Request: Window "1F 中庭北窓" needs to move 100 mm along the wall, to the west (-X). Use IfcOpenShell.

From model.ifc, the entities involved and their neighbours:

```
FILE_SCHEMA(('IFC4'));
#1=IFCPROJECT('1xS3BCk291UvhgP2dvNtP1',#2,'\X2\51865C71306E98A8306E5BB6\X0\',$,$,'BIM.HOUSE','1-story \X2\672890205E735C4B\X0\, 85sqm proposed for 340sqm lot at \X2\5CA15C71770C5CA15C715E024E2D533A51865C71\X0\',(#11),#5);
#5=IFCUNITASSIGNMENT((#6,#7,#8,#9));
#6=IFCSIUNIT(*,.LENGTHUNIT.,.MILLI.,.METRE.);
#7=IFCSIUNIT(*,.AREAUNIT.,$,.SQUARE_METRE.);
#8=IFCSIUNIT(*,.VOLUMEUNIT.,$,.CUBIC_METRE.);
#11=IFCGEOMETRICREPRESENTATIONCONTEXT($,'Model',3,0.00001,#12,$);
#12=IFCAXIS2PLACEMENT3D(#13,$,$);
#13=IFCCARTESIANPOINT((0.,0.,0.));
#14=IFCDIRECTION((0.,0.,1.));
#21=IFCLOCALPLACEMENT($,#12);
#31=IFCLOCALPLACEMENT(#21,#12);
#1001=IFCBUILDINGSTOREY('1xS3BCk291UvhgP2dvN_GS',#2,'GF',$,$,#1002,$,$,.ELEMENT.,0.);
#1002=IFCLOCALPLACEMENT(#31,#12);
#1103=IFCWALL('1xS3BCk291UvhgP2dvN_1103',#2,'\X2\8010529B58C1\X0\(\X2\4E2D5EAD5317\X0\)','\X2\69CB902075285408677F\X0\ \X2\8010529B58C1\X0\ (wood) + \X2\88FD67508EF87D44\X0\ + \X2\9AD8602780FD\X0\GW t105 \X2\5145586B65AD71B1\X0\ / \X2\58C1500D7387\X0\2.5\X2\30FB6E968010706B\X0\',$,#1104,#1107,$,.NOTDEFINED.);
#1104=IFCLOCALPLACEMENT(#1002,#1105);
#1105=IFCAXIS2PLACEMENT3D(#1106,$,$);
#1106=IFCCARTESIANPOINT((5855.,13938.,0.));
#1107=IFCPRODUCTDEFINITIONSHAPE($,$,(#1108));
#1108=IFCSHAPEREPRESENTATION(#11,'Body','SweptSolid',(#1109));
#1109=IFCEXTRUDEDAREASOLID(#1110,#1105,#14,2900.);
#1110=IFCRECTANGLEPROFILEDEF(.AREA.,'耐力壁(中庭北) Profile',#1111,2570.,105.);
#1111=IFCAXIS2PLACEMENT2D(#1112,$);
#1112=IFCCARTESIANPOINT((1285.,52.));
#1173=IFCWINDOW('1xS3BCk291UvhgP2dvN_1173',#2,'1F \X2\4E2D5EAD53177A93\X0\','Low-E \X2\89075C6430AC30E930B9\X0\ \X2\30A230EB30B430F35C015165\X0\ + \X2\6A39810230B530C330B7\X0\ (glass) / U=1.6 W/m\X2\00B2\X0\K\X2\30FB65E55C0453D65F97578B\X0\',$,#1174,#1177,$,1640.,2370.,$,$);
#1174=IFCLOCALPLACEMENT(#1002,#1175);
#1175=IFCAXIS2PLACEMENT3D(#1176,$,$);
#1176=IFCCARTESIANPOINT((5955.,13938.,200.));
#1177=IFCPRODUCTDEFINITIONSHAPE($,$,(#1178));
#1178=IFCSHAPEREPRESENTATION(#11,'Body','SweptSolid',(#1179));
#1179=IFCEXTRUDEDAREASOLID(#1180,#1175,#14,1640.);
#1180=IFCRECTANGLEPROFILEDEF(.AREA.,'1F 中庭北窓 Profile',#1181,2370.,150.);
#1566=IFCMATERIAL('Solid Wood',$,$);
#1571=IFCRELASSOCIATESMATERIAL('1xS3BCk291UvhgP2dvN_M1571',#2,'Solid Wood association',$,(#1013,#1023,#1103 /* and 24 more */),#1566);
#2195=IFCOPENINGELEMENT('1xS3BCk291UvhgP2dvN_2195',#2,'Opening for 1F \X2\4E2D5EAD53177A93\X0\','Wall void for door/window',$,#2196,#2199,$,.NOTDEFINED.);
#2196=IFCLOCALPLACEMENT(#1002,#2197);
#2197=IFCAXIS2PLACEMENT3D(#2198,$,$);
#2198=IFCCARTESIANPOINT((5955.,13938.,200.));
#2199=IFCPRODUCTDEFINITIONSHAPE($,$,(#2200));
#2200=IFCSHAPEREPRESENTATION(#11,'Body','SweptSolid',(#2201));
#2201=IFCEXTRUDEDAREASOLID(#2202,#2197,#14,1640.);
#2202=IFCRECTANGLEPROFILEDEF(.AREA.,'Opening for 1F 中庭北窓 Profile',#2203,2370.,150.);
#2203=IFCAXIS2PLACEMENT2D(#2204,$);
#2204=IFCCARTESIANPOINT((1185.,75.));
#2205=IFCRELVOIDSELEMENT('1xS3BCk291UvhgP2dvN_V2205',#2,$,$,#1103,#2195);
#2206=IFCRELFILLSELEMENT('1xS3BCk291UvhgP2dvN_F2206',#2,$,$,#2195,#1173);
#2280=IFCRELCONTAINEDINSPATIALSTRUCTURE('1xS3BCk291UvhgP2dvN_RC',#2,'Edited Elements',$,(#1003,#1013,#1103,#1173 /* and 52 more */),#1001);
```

```python
import ifcopenshell
import ifcopenshell.api.geometry
import ifcopenshell.util.placement
import ifcopenshell.util.unit

model = ifcopenshell.open("model.ifc")
unit_scale = ifcopenshell.util.unit.calculate_unit_scale(model)

window = model.by_guid("1xS3BCk291UvhgP2dvN_1173")
opening = window.FillsVoids[0].RelatingOpeningElement
wall = opening.VoidsElements[0].RelatingBuildingElement

wall_matrix = ifcopenshell.util.placement.get_local_placement(wall.ObjectPlacement)
shift = wall_matrix[:3, 0] * -0.1 / unit_scale
before = ifcopenshell.util.placement.get_local_placement(window.ObjectPlacement)[:3, 3].copy()

# The window is not placed relative to its opening, so move both.
for product in (opening, window):
    matrix = ifcopenshell.util.placement.get_local_placement(product.ObjectPlacement)
    matrix[:3, 3] += shift
    ifcopenshell.api.geometry.edit_object_placement(model, product=product, matrix=matrix, is_si=False)

after = ifcopenshell.util.placement.get_local_placement(window.ObjectPlacement)[:3, 3]
print("window moved by", (after - before).round(3) + 0.0)

model.write("model_updated.ifc")
```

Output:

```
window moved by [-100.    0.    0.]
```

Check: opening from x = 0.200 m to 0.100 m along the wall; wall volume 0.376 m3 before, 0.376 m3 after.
